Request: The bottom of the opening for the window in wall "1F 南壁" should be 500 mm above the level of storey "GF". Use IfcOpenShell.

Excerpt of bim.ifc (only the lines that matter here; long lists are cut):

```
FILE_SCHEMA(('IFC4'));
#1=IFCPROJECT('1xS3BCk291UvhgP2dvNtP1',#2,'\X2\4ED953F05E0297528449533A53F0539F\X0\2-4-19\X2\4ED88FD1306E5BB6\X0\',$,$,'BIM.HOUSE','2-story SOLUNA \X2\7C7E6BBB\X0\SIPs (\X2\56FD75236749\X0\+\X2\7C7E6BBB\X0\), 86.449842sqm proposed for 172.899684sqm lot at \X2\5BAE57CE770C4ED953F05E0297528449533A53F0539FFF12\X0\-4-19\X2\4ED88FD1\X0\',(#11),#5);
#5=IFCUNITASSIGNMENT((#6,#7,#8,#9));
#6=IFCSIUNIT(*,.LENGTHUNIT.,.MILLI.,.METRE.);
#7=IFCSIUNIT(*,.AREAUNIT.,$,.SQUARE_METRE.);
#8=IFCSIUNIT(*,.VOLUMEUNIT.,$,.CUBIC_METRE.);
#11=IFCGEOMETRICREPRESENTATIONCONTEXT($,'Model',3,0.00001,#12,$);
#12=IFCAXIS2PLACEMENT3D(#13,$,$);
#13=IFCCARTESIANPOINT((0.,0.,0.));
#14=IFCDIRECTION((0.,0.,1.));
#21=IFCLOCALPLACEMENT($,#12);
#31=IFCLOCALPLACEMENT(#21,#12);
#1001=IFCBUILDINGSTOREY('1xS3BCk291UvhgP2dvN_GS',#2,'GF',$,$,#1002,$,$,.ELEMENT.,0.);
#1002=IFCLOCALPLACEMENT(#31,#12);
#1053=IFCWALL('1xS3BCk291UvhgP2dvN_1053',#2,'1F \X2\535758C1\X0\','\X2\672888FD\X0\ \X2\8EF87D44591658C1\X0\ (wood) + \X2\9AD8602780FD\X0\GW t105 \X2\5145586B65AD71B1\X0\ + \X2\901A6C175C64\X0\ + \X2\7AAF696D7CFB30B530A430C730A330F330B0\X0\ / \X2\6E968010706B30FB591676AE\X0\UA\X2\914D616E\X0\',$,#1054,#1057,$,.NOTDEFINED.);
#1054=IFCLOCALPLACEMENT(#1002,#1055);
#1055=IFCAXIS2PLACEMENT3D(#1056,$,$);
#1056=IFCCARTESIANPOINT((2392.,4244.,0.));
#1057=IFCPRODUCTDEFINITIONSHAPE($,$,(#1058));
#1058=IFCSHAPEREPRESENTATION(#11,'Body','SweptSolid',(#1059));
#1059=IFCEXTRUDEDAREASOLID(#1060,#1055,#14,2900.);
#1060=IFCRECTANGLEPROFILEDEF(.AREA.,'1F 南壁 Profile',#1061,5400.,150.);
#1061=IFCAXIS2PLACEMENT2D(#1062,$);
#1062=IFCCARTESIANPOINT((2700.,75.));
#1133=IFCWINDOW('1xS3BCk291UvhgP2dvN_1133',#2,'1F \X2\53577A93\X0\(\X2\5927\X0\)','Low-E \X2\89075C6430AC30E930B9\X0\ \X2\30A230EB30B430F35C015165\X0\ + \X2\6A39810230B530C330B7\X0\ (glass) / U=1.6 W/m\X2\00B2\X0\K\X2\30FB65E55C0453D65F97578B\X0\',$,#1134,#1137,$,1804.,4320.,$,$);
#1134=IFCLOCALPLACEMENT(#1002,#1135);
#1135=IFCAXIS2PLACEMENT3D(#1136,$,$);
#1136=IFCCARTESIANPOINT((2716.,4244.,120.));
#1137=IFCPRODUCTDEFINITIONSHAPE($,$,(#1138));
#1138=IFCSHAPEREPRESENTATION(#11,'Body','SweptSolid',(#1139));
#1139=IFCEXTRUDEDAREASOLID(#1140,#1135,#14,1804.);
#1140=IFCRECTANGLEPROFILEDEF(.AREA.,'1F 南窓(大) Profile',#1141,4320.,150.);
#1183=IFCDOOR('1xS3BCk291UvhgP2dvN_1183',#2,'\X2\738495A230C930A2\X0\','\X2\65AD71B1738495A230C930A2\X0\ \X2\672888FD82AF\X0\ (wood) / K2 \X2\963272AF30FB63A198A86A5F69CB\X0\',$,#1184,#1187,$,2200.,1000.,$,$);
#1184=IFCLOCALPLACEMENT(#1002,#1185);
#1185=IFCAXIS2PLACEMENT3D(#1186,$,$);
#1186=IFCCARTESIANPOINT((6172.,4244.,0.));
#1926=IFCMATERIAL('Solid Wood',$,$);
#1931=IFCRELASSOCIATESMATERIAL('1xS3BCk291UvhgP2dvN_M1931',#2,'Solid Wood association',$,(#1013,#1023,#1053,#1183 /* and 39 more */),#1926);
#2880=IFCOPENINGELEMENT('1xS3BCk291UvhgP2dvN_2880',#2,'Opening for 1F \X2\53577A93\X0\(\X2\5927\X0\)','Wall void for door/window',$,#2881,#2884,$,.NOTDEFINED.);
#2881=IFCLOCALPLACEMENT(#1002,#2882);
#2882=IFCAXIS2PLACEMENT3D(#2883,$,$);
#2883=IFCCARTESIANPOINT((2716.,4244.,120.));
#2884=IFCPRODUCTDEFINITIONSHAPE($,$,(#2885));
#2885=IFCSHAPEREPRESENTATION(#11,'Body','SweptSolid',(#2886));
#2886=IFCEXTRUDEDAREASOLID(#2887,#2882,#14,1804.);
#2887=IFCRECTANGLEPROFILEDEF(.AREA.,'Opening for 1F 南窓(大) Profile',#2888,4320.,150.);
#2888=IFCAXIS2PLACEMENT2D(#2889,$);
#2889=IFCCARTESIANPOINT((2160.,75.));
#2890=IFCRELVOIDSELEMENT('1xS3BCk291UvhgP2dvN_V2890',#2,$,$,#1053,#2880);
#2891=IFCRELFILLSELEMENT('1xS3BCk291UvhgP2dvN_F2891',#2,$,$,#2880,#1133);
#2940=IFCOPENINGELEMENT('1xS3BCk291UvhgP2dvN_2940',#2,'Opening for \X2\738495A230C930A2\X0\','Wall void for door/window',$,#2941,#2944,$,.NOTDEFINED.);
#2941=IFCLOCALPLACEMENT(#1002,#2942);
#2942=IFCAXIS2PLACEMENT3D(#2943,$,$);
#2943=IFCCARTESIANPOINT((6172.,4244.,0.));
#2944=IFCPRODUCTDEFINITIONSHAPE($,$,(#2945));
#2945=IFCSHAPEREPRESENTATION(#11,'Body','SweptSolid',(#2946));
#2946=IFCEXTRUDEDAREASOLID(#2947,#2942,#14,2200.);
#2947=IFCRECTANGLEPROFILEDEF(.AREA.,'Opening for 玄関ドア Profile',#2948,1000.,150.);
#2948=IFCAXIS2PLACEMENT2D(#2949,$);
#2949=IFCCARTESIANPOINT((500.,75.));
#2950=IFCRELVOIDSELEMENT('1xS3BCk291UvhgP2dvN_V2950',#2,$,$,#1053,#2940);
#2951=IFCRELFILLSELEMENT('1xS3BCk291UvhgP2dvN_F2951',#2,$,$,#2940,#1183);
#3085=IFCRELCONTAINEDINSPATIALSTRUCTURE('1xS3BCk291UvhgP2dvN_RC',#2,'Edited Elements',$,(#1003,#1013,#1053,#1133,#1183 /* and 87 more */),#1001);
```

```python
import numpy as np
import ifcopenshell
import ifcopenshell.api.geometry
import ifcopenshell.geom
import ifcopenshell.util.element
import ifcopenshell.util.placement
import ifcopenshell.util.shape
import ifcopenshell.util.unit

model = ifcopenshell.open("bim.ifc")
unit_scale = ifcopenshell.util.unit.calculate_unit_scale(model)

window = model.by_id(1133)
opening = window.FillsVoids[0].RelatingOpeningElement
storey = ifcopenshell.util.element.get_container(window, ifc_class="IfcBuildingStorey")
level = ifcopenshell.util.placement.get_local_placement(storey.ObjectPlacement)[2, 3]

# The opening's origin need not be at the sill, so measure its lowest point.
shape = ifcopenshell.geom.create_shape(ifcopenshell.geom.settings(), opening)
bottom = ifcopenshell.util.shape.get_shape_bottom_elevation(shape, shape.geometry) / unit_scale
dz = level + 0.5 / unit_scale - bottom

shift = np.array([0.0, 0.0, dz])
# The window is not placed relative to its opening, so move both.
for product in (opening, window):
    matrix = ifcopenshell.util.placement.get_local_placement(product.ObjectPlacement)
    matrix[:3, 3] += shift
    ifcopenshell.api.geometry.edit_object_placement(model, product=product, matrix=matrix, is_si=False)

print(f"moved by {dz * unit_scale:+.3f} m")

model.write("bim_updated.ifc")
```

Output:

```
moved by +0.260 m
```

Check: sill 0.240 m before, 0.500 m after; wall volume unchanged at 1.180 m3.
